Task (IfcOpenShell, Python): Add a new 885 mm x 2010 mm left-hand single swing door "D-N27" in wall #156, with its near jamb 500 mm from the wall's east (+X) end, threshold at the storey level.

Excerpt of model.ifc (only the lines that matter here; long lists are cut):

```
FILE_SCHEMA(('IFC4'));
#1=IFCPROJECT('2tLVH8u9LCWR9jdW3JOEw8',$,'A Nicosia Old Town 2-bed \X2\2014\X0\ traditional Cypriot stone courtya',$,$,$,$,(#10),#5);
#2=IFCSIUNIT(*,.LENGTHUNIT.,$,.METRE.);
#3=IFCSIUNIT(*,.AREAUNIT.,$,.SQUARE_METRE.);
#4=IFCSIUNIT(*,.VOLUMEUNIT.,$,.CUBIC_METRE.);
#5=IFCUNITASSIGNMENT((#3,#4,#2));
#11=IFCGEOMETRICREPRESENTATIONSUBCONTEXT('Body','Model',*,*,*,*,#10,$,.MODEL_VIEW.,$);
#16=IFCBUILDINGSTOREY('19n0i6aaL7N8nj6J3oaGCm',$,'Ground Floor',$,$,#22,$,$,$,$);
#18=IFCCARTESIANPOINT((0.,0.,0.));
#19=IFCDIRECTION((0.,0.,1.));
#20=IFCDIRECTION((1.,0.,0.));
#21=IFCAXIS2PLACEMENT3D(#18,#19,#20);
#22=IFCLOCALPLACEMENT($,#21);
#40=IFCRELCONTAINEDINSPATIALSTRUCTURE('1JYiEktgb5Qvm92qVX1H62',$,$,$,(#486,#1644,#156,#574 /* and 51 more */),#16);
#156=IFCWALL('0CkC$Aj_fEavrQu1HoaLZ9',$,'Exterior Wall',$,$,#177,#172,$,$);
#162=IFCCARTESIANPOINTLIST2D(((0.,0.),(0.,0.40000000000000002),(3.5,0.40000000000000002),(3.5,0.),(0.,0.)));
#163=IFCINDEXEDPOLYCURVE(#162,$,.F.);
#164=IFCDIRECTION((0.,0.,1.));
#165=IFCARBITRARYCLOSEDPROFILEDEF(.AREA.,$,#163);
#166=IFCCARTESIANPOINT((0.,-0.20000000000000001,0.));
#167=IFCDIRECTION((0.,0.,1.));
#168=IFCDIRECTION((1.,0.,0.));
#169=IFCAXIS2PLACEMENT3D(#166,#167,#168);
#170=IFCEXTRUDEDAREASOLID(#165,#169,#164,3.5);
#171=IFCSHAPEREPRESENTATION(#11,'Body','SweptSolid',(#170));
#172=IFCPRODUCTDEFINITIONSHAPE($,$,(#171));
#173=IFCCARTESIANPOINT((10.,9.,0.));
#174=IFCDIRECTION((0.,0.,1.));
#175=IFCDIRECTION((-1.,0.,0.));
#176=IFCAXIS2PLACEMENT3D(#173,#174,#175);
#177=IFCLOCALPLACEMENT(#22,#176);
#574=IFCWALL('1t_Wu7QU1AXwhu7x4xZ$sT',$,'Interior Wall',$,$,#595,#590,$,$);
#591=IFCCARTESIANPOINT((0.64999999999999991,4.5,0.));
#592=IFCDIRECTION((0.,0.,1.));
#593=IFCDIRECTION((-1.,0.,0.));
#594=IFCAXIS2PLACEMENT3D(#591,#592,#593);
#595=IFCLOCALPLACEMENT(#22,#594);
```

```python
import numpy as np
import ifcopenshell
import ifcopenshell.api.feature
import ifcopenshell.api.geometry
import ifcopenshell.api.root
import ifcopenshell.api.spatial
import ifcopenshell.geom
import ifcopenshell.util.element
import ifcopenshell.util.placement
import ifcopenshell.util.representation
import ifcopenshell.util.shape
import ifcopenshell.util.unit

model = ifcopenshell.open("model.ifc")
unit_scale = ifcopenshell.util.unit.calculate_unit_scale(model)
settings = ifcopenshell.geom.settings()


def volume(element):
    """Net volume in cubic metres, openings subtracted."""
    shape = ifcopenshell.geom.create_shape(settings, element)
    return ifcopenshell.util.shape.get_volume(shape.geometry)


wall = model.by_id(156)
storey = ifcopenshell.util.element.get_container(wall, ifc_class="IfcBuildingStorey")
context = ifcopenshell.util.representation.get_context(model, "Model", "Body", "MODEL_VIEW")
before = volume(wall)

width, height, from_end, sill = 0.885, 2.01, 0.5, 0.0  # metres

# The wall runs along its own X axis, and the end named is its -X end.
wall_shape = ifcopenshell.geom.create_shape(settings, wall)
x, y, z = ifcopenshell.util.shape.get_vertices(wall_shape.geometry).T
start = x.min() + from_end
face, thickness = float(y.min()), float(y.max() - y.min())
wall_matrix = ifcopenshell.util.placement.get_local_placement(wall.ObjectPlacement)
level = ifcopenshell.util.placement.get_local_placement(storey.ObjectPlacement)[2, 3]


def in_wall(x, y):
    """Placement at x, y metres in the wall's axes, at sill height."""
    matrix = wall_matrix.copy()
    matrix[:, 3] = wall_matrix @ np.array([x / unit_scale, y / unit_scale, 0.0, 1.0])
    matrix[2, 3] = level + sill / unit_scale
    return matrix


# Opening: a box that overshoots both wall faces by 50 mm.
opening = ifcopenshell.api.root.create_entity(model, ifc_class="IfcOpeningElement", predefined_type="OPENING")
box = ifcopenshell.api.geometry.add_wall_representation(
    model, context=context, length=width, height=height, thickness=thickness + 0.1
)
ifcopenshell.api.geometry.assign_representation(model, product=opening, representation=box)
ifcopenshell.api.geometry.edit_object_placement(model, product=opening, matrix=in_wall(start, face - 0.05), is_si=False)
ifcopenshell.api.feature.add_feature(model, feature=opening, element=wall)

door = ifcopenshell.api.root.create_entity(model, ifc_class="IfcDoor", name="D-N27", predefined_type="DOOR")
door.OverallWidth, door.OverallHeight = width / unit_scale, height / unit_scale
door.OperationType = "SINGLE_SWING_LEFT"
body = ifcopenshell.api.geometry.add_door_representation(
    model,
    context=context,
    overall_width=door.OverallWidth,
    overall_height=door.OverallHeight,
    operation_type="SINGLE_SWING_LEFT",
    lining_properties={"LiningDepth": thickness / unit_scale, "ThresholdDepth": thickness / unit_scale},
)
ifcopenshell.api.geometry.assign_representation(model, product=door, representation=body)
ifcopenshell.api.spatial.assign_container(model, products=[door], relating_structure=storey)
ifcopenshell.api.feature.add_filling(model, opening=opening, element=door)

# The lining spans the wall, so the door starts at the wall face.
ifcopenshell.api.geometry.edit_object_placement(model, product=door, matrix=in_wall(start, face), is_si=False)

after = volume(wall)

print(f"wall volume {before:.3f} -> {after:.3f} m3")

model.write("model_edited.ifc")
```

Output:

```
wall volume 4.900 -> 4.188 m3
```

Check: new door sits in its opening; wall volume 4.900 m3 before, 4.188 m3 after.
